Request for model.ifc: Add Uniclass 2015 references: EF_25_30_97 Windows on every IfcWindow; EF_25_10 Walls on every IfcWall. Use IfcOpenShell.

First a look at what the model holds.

```python
import ifcopenshell

model = ifcopenshell.open("model.ifc")
print(model.schema)
print("classifications:", [c.Name for c in model.by_type("IfcClassification")])
for ifc_class in ("IfcDoor", "IfcRoof", "IfcStair", "IfcWall", "IfcWindow"):
    print(ifc_class, len(model.by_type(ifc_class)))
```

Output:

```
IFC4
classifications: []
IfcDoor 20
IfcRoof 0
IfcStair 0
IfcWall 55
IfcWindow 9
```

```python
import ifcopenshell
import ifcopenshell.api.classification

model = ifcopenshell.open("model.ifc")

system = ifcopenshell.api.classification.add_classification(model, classification="Uniclass 2015")

codes = {
    "IfcWindow": ("EF_25_30_97", "Windows"),
    "IfcWall": ("EF_25_10", "Walls"),
}
for ifc_class, (code, name) in codes.items():
    products = model.by_type(ifc_class)
    ifcopenshell.api.classification.add_reference(
        model, products=products, classification=system, identification=code, name=name
    )
    print(code, len(products))

model.write("model_v2.ifc")
```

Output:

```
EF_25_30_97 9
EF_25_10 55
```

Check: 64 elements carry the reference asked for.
